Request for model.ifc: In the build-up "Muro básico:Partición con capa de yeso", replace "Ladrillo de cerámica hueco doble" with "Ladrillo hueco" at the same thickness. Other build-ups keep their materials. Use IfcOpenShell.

First a look at what the model holds.

```python
import ifcopenshell
import ifcopenshell.util.element

model = ifcopenshell.open("model.ifc")
print(model.schema)
for layer_set in model.by_type("IfcMaterialLayerSet"):
    if layer_set.LayerSetName == "Muro básico:Partición con capa de yeso":
        for layer in layer_set.MaterialLayers:
            print(layer.id(), layer.Material and layer.Material.Name, layer.LayerThickness, sep=" | ")
        print(len(ifcopenshell.util.element.get_elements_by_material(model, layer_set)), "elements and types use it")
print(sorted(m.Name for m in model.by_type("IfcMaterial") if m.Name)[:60])
```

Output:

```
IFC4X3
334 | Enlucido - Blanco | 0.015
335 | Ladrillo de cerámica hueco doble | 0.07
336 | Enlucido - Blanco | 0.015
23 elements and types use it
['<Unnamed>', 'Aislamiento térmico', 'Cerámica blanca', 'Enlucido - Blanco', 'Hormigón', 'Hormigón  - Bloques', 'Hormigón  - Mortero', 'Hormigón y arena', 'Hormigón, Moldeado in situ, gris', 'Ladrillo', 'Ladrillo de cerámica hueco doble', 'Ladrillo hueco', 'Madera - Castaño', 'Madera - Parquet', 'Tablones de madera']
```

```python
import ifcopenshell
import ifcopenshell.api.material

model = ifcopenshell.open("model.ifc")

layer_set = next(s for s in model.by_type("IfcMaterialLayerSet") if s.LayerSetName == "Muro básico:Partición con capa de yeso")
layer = next(l for l in layer_set.MaterialLayers if l.Material and l.Material.Name == "Ladrillo de cerámica hueco doble")
material = next(m for m in model.by_type("IfcMaterial") if m.Name == "Ladrillo hueco")

# Point this one layer at the other material; renaming the old one would change it everywhere.
ifcopenshell.api.material.edit_layer(model, layer=layer, attributes={"Name": material.Name}, material=material)

print([l.Material.Name if l.Material else None for l in layer_set.MaterialLayers])

model.write("model_rev.ifc")
```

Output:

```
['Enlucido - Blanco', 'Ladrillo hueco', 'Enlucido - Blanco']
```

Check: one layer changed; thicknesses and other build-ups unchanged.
